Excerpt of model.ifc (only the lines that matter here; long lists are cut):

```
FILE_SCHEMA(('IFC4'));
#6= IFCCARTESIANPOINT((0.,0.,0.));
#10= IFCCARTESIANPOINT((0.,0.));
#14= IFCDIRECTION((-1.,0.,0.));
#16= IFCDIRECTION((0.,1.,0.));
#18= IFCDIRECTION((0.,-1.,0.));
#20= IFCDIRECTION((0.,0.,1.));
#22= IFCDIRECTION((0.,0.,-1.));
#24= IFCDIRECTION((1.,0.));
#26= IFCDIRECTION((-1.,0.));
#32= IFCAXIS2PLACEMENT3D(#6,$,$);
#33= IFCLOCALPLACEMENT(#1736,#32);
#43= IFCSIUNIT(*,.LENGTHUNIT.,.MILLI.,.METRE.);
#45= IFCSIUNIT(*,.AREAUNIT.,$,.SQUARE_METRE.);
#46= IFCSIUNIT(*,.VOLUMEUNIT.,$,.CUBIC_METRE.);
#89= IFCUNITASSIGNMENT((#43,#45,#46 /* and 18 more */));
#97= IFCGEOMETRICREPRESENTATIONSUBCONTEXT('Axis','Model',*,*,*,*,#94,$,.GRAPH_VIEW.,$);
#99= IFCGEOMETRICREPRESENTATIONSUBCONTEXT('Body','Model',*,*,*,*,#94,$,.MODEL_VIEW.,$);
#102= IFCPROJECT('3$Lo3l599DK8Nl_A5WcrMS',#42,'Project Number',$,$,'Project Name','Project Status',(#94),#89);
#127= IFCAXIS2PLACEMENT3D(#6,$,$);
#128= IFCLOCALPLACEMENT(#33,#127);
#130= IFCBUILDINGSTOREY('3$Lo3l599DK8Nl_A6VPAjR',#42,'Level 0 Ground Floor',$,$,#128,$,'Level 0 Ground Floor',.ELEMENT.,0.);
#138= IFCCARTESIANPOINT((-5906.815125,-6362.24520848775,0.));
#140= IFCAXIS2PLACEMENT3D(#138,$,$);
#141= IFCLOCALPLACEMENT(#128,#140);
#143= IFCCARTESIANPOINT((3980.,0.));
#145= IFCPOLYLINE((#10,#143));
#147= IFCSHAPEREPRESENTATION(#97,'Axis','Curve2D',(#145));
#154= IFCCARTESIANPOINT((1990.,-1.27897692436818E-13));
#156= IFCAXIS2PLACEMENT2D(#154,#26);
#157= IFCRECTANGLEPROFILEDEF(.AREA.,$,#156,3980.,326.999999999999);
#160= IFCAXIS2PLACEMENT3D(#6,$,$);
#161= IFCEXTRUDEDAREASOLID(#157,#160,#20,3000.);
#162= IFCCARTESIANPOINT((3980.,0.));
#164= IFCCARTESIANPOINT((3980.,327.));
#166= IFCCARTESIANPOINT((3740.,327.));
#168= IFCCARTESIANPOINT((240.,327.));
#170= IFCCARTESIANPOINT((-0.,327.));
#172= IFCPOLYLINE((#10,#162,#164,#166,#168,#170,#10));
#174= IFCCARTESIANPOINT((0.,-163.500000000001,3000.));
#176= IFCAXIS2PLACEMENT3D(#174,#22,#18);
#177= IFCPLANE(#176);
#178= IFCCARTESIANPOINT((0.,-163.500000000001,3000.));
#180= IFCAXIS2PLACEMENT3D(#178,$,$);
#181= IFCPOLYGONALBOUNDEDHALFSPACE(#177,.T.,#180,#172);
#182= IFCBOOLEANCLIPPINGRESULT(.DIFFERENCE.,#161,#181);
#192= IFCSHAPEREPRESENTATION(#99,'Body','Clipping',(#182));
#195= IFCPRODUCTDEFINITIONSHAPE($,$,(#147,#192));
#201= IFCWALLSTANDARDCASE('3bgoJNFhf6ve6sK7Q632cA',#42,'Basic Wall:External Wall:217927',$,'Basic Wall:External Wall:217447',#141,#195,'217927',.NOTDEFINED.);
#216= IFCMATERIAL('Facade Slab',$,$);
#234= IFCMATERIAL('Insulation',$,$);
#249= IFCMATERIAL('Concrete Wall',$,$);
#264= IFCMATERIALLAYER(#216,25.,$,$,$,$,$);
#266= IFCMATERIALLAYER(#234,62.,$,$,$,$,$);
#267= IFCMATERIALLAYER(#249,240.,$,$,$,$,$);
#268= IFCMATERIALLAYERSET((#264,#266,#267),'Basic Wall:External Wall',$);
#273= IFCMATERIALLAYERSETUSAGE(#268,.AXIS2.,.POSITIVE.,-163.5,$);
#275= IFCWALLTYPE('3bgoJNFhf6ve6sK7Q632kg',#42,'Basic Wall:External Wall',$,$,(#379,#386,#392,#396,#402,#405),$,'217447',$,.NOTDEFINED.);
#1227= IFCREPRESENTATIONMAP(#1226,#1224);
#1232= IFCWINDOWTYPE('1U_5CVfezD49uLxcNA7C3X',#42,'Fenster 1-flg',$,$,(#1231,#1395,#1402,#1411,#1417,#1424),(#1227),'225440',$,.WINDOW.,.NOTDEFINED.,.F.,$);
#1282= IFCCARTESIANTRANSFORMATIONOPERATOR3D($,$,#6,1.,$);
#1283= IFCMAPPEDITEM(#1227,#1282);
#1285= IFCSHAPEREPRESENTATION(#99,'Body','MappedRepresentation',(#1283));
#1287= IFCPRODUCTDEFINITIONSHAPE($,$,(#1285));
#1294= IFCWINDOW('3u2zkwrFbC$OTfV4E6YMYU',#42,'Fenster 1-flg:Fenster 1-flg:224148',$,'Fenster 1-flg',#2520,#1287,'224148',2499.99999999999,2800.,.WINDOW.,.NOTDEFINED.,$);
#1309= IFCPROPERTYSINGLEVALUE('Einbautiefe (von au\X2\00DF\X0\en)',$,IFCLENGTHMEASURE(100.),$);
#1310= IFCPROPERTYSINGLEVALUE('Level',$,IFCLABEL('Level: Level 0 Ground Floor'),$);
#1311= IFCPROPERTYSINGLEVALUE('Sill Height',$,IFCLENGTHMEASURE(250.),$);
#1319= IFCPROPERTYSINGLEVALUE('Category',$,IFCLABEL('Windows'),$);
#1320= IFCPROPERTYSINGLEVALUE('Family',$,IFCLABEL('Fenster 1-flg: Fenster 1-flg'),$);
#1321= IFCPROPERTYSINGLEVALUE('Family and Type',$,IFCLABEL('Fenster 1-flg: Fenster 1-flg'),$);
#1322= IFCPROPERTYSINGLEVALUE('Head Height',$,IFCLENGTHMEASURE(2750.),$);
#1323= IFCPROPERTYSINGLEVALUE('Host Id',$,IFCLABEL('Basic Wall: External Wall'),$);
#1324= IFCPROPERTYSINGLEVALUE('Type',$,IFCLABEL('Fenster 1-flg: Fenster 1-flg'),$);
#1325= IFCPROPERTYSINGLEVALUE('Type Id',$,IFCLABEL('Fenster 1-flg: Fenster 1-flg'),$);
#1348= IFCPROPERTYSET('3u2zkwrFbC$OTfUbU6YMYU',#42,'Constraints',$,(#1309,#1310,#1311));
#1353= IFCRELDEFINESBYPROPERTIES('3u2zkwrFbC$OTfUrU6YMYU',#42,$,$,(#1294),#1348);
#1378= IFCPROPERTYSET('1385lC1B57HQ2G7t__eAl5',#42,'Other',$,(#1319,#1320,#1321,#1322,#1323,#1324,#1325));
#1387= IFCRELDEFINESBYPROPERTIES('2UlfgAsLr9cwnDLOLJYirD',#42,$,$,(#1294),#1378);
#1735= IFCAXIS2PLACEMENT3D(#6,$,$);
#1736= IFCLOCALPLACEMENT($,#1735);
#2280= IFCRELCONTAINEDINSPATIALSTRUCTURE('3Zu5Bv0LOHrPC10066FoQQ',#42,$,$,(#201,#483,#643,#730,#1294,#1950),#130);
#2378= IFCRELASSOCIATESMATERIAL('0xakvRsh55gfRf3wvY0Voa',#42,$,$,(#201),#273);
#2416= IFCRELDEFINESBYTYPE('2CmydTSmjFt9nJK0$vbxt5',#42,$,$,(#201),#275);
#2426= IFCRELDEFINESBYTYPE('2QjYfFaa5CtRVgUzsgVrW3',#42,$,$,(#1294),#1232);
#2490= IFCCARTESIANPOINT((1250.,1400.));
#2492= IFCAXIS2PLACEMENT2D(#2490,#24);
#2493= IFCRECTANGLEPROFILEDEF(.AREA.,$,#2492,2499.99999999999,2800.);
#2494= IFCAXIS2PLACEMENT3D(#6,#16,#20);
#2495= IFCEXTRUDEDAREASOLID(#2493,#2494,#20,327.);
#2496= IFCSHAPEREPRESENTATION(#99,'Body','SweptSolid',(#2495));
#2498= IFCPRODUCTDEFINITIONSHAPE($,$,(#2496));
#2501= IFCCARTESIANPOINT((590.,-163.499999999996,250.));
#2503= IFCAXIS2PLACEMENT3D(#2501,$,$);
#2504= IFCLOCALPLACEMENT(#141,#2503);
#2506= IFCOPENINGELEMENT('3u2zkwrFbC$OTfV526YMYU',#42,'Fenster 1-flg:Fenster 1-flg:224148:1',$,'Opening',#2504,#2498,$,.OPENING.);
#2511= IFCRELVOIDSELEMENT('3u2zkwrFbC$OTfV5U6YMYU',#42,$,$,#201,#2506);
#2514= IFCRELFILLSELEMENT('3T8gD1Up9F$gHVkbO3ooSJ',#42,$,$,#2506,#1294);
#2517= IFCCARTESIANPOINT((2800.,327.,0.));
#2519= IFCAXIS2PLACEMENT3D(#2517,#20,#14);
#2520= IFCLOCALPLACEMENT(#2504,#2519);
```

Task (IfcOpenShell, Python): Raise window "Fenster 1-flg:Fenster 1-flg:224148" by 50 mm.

```python
import numpy as np
import ifcopenshell
import ifcopenshell.api.geometry
import ifcopenshell.api.pset
import ifcopenshell.util.element
import ifcopenshell.util.placement
import ifcopenshell.util.unit

model = ifcopenshell.open("model.ifc")
unit_scale = ifcopenshell.util.unit.calculate_unit_scale(model)

window = model.by_guid("3u2zkwrFbC$OTfV4E6YMYU")
opening = window.FillsVoids[0].RelatingOpeningElement
dz = 0.05 / unit_scale

shift = np.array([0.0, 0.0, dz])
# The window is placed relative to its opening, so it follows when the opening moves.
matrix = ifcopenshell.util.placement.get_local_placement(opening.ObjectPlacement)
matrix[:3, 3] += shift
ifcopenshell.api.geometry.edit_object_placement(
    model, product=opening, matrix=matrix, is_si=False, should_transform_children=True
)

# Keep the stored heights in step.
pset = model.by_id(ifcopenshell.util.element.get_pset(window, "Constraints", should_inherit=False)["id"])
ifcopenshell.api.pset.edit_pset(model, pset=pset, properties={
    "Sill Height": model.create_entity("IfcLengthMeasure", ifcopenshell.util.element.get_pset(window, "Constraints", "Sill Height") + dz),
})
pset = model.by_id(ifcopenshell.util.element.get_pset(window, "Other", should_inherit=False)["id"])
ifcopenshell.api.pset.edit_pset(model, pset=pset, properties={
    "Head Height": model.create_entity("IfcLengthMeasure", ifcopenshell.util.element.get_pset(window, "Other", "Head Height") + dz),
})

print(f"moved by {dz * unit_scale:+.3f} m")

model.write("model_updated.ifc")
```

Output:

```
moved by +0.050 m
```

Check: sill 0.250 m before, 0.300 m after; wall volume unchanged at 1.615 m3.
